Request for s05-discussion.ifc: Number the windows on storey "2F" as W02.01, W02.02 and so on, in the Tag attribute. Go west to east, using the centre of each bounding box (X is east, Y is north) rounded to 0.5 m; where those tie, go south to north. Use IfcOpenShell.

First a look at what the model holds.

```python
import ifcopenshell
import ifcopenshell.util.element
import ifcopenshell.util.placement

model = ifcopenshell.open("s05-discussion.ifc")
print(model.schema)
storey = next(s for s in model.by_type("IfcBuildingStorey") if s.Name == "2F")
windows = [e for e in ifcopenshell.util.element.get_decomposition(storey) if e.is_a("IfcWindow")]
for e in sorted(windows, key=lambda e: e.id()):
    origin = ifcopenshell.util.placement.get_local_placement(e.ObjectPlacement)[:3, 3]
    print(e.id(), e.Tag, e.Name, origin.round(2) + 0.0, sep=" | ")
```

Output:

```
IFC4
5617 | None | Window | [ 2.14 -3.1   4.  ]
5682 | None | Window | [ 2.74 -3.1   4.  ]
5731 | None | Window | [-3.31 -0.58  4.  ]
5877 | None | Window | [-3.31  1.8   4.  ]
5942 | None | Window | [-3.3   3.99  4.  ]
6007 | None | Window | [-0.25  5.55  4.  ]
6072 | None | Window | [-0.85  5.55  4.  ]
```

```python
import ifcopenshell
import ifcopenshell.geom
import ifcopenshell.util.element
import ifcopenshell.util.shape

model = ifcopenshell.open("s05-discussion.ifc")
settings = ifcopenshell.geom.settings()
settings.set("use-world-coords", True)


def centre(element):
    shape = ifcopenshell.geom.create_shape(settings, element)
    return ifcopenshell.util.shape.get_bbox_centroid(shape.geometry)


storey = next(s for s in model.by_type("IfcBuildingStorey") if s.Name == "2F")
windows = [e for e in ifcopenshell.util.element.get_decomposition(storey) if e.is_a("IfcWindow")]

# Insertion points can sit at a corner or the storey origin, so sort by the geometry (in metres).
centres = {e: centre(e) for e in windows}
windows.sort(key=lambda e: (round(centres[e][0] / 0.5), centres[e][1]))

for i, e in enumerate(windows, start=1):
    number = f"W02.{i:02d}"
    e.Tag = number
    print(e.id(), number)

model.write("s05-discussion_rev.ifc")
```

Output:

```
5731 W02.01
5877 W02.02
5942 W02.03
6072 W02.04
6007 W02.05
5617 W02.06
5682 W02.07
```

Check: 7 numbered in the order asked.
